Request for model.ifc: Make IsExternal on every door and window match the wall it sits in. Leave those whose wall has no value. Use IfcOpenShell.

First a look at what the model holds.

```python
import ifcopenshell
import ifcopenshell.util.element

model = ifcopenshell.open("model.ifc")
print(model.schema)
seen = {}
for e in model.by_type("IfcDoor") + model.by_type("IfcWindow"):
    if not e.FillsVoids:
        continue
    host = e.FillsVoids[0].RelatingOpeningElement.VoidsElements[0].RelatingBuildingElement
    own = ifcopenshell.util.element.get_pset(e, f"Pset_{e.is_a()[3:].removesuffix('StandardCase')}Common", "IsExternal")
    wall = ifcopenshell.util.element.get_pset(host, "Pset_WallCommon", "IsExternal")
    seen[e.is_a(), own, wall] = seen.get((e.is_a(), own, wall), 0) + 1
for (cls, own, wall), count in sorted(seen.items(), key=str):
    print(count, cls, "IsExternal:", own, "| host wall:", wall)
```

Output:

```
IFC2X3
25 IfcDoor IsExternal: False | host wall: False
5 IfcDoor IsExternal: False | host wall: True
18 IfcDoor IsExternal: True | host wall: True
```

```python
import ifcopenshell
import ifcopenshell.api.pset
import ifcopenshell.util.element

model = ifcopenshell.open("model.ifc")

count = 0
for ifc_class, pset_name in (("IfcDoor", "Pset_DoorCommon"), ("IfcWindow", "Pset_WindowCommon")):
    for e in model.by_type(ifc_class):
        if not e.FillsVoids:
            continue
        host = e.FillsVoids[0].RelatingOpeningElement.VoidsElements[0].RelatingBuildingElement
        external = ifcopenshell.util.element.get_pset(host, "Pset_WallCommon", "IsExternal")
        if external is None or ifcopenshell.util.element.get_pset(e, pset_name, "IsExternal") == external:
            continue
        pset = ifcopenshell.api.pset.add_pset(model, product=e, name=pset_name)
        ifcopenshell.api.pset.edit_pset(model, pset=pset, properties={"IsExternal": external})
        count += 1

print(count, "updated")

model.write("model_edited.ifc")
```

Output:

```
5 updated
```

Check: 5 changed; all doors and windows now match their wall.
